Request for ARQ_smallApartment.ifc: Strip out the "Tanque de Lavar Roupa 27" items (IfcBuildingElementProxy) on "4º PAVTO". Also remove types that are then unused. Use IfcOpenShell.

First a look at what the model holds.

```python
import ifcopenshell
import ifcopenshell.util.element

model = ifcopenshell.open("ARQ_smallApartment.ifc")
print(model.schema)
storey = next(s for s in model.by_type("IfcBuildingStorey") if s.Name == "4º PAVTO")
proxies = [e for e in ifcopenshell.util.element.get_decomposition(storey) if e.is_a("IfcBuildingElementProxy")]
seen = {}
for e in proxies:
    element_type = ifcopenshell.util.element.get_type(e)
    name = element_type.Name if element_type not in (None, e) else None
    seen[name] = seen.get(name, 0) + 1
for name, count in sorted(seen.items(), key=str):
    print(count, "x", name)
```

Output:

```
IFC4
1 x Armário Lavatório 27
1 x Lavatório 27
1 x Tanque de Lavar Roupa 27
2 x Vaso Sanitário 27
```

```python
import ifcopenshell
import ifcopenshell.api.root
import ifcopenshell.util.element

model = ifcopenshell.open("ARQ_smallApartment.ifc")

storey = next(s for s in model.by_type("IfcBuildingStorey") if s.Name == "4º PAVTO")
proxies = [e for e in ifcopenshell.util.element.get_decomposition(storey) if e.is_a("IfcBuildingElementProxy")]
targets = [e for e in proxies if (t := ifcopenshell.util.element.get_type(e)) not in (None, e) and t.Name == "Tanque de Lavar Roupa 27"]
types = {ifcopenshell.util.element.get_type(e) for e in targets} - {None, *targets}

for e in targets:
    ifcopenshell.api.root.remove_product(model, product=e)
print(len(targets), "removed")

unused = [t for t in types if not ifcopenshell.util.element.get_types(t)]
for t in unused:
    ifcopenshell.api.root.remove_product(model, product=t)
print(len(unused), "unused types removed")

model.write("ARQ_smallApartment_updated.ifc")
```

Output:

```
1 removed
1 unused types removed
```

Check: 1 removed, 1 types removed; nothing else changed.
